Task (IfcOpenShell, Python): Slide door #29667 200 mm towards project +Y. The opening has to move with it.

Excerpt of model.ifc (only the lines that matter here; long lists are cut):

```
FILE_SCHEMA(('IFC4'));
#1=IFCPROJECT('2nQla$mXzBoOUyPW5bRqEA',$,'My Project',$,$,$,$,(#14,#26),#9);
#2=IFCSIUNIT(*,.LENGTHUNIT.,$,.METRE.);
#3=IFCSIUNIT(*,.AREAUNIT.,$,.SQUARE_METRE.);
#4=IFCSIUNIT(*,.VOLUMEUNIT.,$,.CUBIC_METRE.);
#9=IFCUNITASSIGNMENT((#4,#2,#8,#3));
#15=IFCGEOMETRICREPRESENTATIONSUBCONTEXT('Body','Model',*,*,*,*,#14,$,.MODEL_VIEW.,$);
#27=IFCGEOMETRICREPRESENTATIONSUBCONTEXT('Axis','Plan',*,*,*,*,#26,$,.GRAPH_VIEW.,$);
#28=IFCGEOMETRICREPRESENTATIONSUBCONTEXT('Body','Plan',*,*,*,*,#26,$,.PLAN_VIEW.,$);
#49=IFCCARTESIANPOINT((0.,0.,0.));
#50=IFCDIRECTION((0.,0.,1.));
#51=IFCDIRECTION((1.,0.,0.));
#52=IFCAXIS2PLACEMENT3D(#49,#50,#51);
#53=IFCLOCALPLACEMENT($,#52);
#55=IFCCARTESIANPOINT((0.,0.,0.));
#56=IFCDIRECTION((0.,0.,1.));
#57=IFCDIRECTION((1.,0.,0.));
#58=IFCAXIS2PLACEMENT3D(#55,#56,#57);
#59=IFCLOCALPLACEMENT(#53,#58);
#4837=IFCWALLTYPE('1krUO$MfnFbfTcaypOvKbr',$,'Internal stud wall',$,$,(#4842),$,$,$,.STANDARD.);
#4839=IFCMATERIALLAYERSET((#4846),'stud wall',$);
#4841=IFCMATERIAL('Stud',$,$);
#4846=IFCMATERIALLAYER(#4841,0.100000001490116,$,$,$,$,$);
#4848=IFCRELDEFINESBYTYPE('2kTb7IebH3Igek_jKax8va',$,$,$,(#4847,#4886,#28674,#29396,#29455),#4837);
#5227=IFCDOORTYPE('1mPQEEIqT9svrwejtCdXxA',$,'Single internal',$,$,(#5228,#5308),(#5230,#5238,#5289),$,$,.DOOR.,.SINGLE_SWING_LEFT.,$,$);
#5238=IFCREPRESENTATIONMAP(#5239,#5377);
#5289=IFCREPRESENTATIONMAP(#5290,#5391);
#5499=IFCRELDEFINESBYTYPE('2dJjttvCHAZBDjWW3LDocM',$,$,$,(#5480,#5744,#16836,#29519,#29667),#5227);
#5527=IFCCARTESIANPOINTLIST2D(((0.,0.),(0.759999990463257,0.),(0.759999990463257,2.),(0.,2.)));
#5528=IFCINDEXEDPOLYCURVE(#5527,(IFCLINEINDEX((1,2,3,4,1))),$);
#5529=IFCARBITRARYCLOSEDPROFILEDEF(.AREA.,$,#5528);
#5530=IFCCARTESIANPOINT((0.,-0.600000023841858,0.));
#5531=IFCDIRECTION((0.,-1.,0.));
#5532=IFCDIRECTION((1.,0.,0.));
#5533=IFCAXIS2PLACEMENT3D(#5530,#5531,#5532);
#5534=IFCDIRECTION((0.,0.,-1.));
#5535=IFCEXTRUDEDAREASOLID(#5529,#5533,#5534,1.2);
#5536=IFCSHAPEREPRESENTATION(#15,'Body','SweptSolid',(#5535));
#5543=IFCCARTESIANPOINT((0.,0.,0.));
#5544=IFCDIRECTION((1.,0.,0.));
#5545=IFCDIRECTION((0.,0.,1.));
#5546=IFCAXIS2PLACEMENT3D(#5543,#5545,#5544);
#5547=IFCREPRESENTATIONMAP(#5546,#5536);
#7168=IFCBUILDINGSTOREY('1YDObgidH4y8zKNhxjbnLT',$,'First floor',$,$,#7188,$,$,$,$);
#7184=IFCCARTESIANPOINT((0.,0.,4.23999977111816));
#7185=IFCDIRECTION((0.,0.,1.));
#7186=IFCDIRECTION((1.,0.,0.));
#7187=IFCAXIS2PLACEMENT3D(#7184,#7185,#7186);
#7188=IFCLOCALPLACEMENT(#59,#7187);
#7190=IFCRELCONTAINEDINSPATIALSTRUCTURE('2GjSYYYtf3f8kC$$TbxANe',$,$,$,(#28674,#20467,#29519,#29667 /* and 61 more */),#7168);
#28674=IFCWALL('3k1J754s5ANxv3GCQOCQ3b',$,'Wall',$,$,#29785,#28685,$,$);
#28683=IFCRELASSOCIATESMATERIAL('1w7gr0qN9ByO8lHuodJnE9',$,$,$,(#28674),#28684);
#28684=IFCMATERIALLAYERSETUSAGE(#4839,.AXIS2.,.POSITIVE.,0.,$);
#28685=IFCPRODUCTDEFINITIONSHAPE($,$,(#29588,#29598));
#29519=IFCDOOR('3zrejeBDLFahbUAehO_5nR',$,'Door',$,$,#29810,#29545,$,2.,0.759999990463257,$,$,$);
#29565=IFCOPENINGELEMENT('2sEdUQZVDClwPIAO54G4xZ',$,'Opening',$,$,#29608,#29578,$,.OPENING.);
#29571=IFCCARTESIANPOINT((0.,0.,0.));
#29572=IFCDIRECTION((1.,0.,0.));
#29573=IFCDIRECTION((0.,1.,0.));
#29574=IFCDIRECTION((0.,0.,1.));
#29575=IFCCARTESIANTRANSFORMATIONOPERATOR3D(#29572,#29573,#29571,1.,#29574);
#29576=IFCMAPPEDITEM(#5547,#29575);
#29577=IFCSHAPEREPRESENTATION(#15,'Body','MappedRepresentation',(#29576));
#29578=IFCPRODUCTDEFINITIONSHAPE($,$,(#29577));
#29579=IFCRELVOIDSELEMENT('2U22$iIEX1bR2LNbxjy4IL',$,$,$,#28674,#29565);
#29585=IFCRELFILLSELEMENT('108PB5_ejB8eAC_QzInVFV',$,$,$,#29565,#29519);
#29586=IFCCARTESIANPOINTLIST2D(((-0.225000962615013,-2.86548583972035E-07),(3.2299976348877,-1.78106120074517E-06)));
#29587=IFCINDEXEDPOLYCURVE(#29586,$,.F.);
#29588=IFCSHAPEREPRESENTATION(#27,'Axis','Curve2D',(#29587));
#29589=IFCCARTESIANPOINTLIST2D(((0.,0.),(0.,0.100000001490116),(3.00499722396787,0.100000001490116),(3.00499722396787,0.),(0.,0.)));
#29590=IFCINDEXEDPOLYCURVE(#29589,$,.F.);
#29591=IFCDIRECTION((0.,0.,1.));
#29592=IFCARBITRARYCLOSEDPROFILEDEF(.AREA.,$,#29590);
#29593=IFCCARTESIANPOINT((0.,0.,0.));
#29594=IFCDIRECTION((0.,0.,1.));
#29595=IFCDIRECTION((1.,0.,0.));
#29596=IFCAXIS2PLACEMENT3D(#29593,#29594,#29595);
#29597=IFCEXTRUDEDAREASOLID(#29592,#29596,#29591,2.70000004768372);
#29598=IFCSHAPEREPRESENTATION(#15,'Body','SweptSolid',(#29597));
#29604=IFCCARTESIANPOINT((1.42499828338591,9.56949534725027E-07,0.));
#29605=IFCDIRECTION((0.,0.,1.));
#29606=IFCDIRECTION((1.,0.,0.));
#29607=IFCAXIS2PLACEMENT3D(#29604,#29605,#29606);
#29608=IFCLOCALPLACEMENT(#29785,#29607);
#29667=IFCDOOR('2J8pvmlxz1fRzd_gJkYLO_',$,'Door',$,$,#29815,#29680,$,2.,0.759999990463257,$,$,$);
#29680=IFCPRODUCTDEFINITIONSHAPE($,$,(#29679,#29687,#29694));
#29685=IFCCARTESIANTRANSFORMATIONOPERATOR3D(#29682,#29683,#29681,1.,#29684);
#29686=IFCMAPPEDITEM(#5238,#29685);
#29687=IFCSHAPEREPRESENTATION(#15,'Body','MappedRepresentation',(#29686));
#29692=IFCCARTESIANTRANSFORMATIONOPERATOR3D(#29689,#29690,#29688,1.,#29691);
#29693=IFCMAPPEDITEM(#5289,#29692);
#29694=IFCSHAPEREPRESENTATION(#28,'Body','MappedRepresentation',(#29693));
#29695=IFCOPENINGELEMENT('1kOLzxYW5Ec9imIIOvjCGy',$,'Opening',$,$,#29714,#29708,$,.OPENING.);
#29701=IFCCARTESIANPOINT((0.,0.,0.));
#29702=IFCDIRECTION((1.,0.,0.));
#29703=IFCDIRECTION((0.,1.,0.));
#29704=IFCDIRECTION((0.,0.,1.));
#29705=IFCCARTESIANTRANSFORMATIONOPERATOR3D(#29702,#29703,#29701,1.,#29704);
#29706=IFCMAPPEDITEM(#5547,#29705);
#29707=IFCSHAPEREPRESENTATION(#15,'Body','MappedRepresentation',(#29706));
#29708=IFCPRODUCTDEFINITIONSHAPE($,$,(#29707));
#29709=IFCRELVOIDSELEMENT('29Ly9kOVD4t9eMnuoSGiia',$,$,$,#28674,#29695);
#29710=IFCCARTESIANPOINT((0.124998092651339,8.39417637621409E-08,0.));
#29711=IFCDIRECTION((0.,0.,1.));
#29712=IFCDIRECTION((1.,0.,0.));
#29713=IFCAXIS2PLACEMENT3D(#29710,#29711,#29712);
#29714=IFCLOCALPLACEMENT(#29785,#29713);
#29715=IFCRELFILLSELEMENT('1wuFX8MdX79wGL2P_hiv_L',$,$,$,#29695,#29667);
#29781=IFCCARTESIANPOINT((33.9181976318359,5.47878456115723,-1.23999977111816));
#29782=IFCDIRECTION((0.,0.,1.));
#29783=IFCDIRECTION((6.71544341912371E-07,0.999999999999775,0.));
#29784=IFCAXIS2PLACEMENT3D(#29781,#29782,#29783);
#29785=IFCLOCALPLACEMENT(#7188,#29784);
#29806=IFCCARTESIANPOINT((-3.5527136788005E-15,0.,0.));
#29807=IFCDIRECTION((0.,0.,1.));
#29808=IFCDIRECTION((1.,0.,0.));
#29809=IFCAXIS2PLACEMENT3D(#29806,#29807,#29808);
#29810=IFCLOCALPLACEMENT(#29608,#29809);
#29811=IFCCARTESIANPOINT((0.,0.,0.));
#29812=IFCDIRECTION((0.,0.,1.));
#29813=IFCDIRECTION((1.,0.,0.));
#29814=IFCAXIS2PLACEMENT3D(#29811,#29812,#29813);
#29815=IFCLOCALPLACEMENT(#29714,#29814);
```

```python
import ifcopenshell
import ifcopenshell.api.geometry
import ifcopenshell.util.placement
import ifcopenshell.util.unit

model = ifcopenshell.open("model.ifc")
unit_scale = ifcopenshell.util.unit.calculate_unit_scale(model)

door = model.by_guid("2J8pvmlxz1fRzd_gJkYLO_")
opening = door.FillsVoids[0].RelatingOpeningElement
wall = opening.VoidsElements[0].RelatingBuildingElement

wall_matrix = ifcopenshell.util.placement.get_local_placement(wall.ObjectPlacement)
shift = wall_matrix[:3, 0] * 0.2 / unit_scale
before = ifcopenshell.util.placement.get_local_placement(door.ObjectPlacement)[:3, 3].copy()

# The door is placed relative to its opening, so it follows when the opening moves.
matrix = ifcopenshell.util.placement.get_local_placement(opening.ObjectPlacement)
matrix[:3, 3] += shift
ifcopenshell.api.geometry.edit_object_placement(
    model, product=opening, matrix=matrix, is_si=False, should_transform_children=True
)

after = ifcopenshell.util.placement.get_local_placement(door.ObjectPlacement)[:3, 3]
print("door moved by", (after - before).round(3) + 0.0)

model.write("model-out.ifc")
```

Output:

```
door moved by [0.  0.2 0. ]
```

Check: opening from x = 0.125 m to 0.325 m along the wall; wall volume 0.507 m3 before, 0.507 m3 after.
